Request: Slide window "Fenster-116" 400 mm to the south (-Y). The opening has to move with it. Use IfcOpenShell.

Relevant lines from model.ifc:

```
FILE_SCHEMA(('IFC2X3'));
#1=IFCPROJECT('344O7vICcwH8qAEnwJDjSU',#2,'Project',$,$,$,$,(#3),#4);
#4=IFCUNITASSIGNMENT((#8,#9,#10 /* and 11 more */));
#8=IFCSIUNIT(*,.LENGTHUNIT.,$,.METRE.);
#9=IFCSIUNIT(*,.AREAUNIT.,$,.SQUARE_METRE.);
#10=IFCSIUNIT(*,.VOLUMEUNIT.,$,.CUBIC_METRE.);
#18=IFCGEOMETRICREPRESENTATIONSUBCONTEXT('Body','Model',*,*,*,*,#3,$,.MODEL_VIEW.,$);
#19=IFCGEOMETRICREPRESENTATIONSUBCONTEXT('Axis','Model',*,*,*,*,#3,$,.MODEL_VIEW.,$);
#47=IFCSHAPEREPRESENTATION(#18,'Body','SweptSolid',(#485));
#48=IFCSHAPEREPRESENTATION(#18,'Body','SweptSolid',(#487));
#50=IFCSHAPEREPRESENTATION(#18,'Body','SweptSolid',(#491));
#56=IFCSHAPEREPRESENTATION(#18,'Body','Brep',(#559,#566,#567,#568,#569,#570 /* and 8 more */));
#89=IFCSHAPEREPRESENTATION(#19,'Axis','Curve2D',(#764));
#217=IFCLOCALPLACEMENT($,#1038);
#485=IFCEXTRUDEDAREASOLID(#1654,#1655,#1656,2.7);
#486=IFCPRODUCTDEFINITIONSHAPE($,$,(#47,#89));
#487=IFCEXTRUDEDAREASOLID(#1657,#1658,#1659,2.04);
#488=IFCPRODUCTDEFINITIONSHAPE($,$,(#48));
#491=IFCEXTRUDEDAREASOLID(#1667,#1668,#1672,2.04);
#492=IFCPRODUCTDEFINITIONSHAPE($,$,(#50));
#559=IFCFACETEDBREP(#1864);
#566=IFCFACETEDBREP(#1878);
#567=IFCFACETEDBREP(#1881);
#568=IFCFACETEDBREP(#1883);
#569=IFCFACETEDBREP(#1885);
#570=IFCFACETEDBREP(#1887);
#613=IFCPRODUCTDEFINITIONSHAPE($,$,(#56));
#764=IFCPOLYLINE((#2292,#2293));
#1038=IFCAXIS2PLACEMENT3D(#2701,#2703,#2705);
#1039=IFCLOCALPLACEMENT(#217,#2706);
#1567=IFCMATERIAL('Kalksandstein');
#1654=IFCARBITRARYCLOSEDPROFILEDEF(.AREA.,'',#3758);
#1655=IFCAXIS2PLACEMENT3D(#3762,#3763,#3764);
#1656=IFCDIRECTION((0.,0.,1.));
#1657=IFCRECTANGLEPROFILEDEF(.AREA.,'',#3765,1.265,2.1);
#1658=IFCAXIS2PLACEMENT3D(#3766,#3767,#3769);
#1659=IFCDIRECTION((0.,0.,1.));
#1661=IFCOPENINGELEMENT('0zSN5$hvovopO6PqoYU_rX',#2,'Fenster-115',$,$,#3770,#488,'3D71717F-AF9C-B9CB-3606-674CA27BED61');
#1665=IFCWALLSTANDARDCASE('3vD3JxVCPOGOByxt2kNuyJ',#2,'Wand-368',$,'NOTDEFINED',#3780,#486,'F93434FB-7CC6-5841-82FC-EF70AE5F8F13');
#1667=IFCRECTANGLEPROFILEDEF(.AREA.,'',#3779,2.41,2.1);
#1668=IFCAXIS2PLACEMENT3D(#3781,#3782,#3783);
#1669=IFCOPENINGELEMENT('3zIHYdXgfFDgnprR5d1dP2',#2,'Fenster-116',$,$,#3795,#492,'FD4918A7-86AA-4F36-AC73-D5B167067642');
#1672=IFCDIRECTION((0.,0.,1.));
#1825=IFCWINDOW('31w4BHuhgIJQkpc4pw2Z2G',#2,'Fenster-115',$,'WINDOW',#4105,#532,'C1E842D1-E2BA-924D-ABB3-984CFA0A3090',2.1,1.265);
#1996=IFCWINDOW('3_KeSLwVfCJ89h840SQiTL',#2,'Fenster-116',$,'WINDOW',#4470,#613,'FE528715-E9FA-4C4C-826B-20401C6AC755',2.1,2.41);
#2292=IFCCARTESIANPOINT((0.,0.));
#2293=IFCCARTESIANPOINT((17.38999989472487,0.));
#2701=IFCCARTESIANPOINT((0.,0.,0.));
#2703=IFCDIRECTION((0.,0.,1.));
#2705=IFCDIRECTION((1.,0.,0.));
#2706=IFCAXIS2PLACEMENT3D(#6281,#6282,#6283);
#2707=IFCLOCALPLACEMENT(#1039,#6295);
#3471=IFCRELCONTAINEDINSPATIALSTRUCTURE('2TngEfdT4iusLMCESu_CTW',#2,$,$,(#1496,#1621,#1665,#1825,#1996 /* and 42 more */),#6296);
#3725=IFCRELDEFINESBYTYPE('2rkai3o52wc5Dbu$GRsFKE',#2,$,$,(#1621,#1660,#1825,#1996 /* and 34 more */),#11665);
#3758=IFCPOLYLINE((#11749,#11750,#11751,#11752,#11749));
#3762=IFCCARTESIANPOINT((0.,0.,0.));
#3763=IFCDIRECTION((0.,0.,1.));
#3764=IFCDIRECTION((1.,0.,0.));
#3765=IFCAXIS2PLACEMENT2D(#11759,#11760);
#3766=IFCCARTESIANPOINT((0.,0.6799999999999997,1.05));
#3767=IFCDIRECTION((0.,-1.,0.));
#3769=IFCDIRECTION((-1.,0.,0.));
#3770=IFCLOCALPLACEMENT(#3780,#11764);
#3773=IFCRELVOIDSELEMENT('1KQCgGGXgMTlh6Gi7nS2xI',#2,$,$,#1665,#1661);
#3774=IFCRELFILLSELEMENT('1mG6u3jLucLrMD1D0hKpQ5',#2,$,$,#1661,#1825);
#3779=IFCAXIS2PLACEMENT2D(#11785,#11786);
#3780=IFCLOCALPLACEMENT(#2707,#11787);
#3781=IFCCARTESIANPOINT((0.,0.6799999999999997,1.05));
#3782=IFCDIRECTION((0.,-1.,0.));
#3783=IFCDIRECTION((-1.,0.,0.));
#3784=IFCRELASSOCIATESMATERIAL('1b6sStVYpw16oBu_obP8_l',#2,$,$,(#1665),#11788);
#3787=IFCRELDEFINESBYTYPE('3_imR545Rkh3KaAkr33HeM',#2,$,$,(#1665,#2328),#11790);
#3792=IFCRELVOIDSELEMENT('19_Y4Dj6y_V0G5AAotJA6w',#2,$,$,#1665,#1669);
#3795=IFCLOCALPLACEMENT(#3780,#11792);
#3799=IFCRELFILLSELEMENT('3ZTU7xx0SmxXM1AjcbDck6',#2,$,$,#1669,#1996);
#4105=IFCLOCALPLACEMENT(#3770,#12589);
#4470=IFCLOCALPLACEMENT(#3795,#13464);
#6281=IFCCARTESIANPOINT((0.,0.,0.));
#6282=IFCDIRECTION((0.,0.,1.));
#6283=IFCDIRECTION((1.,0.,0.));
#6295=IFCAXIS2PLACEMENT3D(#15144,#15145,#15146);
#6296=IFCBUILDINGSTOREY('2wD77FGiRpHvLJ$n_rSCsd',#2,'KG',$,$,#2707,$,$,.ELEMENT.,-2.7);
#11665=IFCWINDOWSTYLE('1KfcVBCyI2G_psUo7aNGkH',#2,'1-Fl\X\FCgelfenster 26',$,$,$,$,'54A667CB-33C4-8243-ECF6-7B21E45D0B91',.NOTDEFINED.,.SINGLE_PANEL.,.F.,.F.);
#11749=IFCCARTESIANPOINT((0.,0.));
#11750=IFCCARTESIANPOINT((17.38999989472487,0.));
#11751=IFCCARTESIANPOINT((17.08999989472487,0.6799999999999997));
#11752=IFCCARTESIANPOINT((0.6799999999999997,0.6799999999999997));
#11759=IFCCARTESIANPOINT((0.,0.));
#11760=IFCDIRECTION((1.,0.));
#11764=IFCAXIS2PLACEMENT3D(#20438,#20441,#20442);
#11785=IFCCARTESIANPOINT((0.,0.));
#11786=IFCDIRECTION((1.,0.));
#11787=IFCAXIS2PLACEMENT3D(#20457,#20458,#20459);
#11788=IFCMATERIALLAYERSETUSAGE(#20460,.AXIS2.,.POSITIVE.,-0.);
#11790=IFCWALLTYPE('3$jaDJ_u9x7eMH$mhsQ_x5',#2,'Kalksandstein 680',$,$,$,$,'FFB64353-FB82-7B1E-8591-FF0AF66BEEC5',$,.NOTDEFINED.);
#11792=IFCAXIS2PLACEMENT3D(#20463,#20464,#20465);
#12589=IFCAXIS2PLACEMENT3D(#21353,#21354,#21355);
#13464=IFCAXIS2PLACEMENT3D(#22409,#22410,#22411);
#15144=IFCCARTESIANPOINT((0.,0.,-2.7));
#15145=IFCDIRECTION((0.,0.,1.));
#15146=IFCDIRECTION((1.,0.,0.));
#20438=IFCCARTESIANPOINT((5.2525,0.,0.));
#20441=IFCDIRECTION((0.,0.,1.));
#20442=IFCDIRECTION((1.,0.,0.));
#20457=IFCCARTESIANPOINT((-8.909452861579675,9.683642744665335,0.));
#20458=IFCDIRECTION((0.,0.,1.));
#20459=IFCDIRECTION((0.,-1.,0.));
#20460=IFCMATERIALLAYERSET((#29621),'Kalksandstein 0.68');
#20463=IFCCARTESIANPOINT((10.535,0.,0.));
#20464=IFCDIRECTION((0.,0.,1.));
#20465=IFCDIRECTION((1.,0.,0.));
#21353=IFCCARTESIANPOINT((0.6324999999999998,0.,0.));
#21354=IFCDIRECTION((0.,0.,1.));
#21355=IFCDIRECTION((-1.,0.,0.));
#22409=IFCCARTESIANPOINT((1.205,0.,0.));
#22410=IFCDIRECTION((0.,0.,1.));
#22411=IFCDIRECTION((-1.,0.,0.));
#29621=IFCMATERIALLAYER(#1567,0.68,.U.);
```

```python
import ifcopenshell
import ifcopenshell.api.geometry
import ifcopenshell.util.placement

model = ifcopenshell.open("model.ifc")

window = model.by_guid("3_KeSLwVfCJ89h840SQiTL")
opening = window.FillsVoids[0].RelatingOpeningElement
wall = opening.VoidsElements[0].RelatingBuildingElement

wall_matrix = ifcopenshell.util.placement.get_local_placement(wall.ObjectPlacement)
shift = wall_matrix[:3, 0] * 0.4
before = ifcopenshell.util.placement.get_local_placement(window.ObjectPlacement)[:3, 3].copy()

# The window is placed relative to its opening, so it follows when the opening moves.
matrix = ifcopenshell.util.placement.get_local_placement(opening.ObjectPlacement)
matrix[:3, 3] += shift
ifcopenshell.api.geometry.edit_object_placement(
    model, product=opening, matrix=matrix, is_si=False, should_transform_children=True
)

after = ifcopenshell.util.placement.get_local_placement(window.ObjectPlacement)[:3, 3]
print("window moved by", (after - before).round(3) + 0.0)

model.write("model_rev.ifc")
```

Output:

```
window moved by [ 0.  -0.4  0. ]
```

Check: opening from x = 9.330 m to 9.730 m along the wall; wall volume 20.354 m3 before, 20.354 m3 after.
